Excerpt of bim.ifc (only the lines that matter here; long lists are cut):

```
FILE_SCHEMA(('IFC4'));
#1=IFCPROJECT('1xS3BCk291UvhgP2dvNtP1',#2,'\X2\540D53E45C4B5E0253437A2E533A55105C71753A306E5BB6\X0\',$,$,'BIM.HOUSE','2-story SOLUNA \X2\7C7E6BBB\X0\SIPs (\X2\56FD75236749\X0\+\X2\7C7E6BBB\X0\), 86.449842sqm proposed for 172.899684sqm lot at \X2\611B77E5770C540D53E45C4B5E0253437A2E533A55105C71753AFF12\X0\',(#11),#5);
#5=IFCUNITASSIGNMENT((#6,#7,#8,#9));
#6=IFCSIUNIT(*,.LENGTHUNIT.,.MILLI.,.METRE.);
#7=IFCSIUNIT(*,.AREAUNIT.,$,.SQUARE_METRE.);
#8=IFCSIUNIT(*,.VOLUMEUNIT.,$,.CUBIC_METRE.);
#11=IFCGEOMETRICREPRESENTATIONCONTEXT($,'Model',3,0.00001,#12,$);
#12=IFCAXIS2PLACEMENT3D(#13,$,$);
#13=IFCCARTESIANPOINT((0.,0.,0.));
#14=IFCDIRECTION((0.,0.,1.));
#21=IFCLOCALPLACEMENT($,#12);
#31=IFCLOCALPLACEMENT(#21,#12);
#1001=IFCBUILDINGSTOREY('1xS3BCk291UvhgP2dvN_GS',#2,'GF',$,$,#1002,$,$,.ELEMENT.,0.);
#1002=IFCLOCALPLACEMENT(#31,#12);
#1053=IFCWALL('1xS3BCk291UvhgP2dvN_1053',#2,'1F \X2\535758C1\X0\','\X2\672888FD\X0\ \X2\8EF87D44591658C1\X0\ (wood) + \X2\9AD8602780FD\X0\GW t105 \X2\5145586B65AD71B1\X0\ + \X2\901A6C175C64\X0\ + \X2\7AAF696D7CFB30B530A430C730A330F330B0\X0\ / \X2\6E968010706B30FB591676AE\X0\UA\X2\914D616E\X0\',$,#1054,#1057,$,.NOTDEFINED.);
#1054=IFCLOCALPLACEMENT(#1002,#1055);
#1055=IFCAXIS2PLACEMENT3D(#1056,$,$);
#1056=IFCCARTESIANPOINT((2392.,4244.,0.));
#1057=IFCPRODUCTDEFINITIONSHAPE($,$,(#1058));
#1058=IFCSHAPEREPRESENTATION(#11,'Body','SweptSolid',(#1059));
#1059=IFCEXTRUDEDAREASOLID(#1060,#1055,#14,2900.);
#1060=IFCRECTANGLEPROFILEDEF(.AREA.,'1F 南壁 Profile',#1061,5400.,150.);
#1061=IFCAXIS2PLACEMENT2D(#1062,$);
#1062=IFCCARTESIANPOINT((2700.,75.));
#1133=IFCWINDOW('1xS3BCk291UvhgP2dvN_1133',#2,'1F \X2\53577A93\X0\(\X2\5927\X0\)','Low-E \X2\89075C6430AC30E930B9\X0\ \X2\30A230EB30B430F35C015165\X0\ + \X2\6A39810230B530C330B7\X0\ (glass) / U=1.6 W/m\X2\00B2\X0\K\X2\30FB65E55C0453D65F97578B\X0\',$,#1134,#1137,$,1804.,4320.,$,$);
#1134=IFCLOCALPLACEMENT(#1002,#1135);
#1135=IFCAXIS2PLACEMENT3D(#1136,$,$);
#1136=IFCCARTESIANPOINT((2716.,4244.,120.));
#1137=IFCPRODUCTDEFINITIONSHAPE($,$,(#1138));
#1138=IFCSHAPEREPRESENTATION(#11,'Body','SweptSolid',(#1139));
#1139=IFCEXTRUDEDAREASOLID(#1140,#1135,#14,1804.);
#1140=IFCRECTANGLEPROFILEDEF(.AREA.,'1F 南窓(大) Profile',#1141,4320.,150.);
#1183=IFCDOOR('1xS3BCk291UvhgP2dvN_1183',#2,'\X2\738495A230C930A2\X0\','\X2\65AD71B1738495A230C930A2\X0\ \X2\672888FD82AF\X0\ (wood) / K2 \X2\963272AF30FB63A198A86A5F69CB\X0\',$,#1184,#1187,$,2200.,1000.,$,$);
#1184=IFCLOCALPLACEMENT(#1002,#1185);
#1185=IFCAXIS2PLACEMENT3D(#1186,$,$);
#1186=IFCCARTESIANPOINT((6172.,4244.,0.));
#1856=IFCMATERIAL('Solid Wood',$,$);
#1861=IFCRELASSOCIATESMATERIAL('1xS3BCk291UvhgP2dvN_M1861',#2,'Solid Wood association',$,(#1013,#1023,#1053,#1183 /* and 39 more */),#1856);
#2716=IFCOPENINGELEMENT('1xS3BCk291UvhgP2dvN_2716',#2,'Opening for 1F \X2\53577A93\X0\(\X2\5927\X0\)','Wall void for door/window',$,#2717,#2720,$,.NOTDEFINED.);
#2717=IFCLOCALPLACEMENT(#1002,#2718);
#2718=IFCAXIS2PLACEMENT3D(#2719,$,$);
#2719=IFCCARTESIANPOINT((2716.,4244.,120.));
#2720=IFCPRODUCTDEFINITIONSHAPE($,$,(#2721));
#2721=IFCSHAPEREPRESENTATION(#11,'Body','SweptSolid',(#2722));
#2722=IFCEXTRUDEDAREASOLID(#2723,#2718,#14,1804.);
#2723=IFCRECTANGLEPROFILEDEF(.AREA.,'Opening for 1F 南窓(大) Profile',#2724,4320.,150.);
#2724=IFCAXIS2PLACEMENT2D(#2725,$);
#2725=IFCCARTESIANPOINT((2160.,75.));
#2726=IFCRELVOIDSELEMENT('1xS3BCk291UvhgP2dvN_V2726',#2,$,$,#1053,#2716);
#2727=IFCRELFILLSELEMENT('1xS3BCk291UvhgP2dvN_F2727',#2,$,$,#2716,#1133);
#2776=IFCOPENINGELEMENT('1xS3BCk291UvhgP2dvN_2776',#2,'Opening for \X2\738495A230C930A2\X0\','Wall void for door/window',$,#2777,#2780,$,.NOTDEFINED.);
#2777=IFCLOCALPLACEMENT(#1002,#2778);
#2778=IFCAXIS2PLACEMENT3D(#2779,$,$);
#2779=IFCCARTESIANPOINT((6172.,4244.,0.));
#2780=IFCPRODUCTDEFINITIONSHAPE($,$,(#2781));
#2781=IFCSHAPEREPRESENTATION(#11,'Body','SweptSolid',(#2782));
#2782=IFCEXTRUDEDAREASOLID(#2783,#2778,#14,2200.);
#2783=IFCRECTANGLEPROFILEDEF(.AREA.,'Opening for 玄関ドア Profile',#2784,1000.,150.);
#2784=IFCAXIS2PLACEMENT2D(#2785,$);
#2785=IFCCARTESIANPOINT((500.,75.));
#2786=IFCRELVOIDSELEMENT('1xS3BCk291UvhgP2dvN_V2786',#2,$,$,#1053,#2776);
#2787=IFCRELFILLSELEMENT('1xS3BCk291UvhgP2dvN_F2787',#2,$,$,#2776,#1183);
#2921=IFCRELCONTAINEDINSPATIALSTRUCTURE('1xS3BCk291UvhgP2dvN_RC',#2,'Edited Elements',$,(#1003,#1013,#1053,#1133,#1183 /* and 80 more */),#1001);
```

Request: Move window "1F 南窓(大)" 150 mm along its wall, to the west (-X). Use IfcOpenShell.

```python
import ifcopenshell
import ifcopenshell.api.geometry
import ifcopenshell.util.placement

model = ifcopenshell.open("bim.ifc")

window = model.by_guid("1xS3BCk291UvhgP2dvN_1133")
opening = window.FillsVoids[0].RelatingOpeningElement
wall = opening.VoidsElements[0].RelatingBuildingElement

wall_matrix = ifcopenshell.util.placement.get_local_placement(wall.ObjectPlacement)
shift = wall_matrix[:3, 0] * -150.0
before = ifcopenshell.util.placement.get_local_placement(window.ObjectPlacement)[:3, 3].copy()

# The window is not placed relative to its opening, so move both.
for product in (opening, window):
    matrix = ifcopenshell.util.placement.get_local_placement(product.ObjectPlacement)
    matrix[:3, 3] += shift
    ifcopenshell.api.geometry.edit_object_placement(model, product=product, matrix=matrix, is_si=False)

after = ifcopenshell.util.placement.get_local_placement(window.ObjectPlacement)[:3, 3]
print("window moved by", (after - before).round(3) + 0.0)

model.write("bim-out.ifc")
```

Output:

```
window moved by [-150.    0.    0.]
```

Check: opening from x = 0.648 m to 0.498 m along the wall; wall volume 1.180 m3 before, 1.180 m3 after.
